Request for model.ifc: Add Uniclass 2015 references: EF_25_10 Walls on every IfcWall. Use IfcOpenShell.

First a look at what the model holds.

```python
import ifcopenshell

model = ifcopenshell.open("model.ifc")
print(model.schema)
print("classifications:", [c.Name for c in model.by_type("IfcClassification")])
for ifc_class in ("IfcDoor", "IfcRoof", "IfcStair", "IfcWall", "IfcWindow"):
    print(ifc_class, len(model.by_type(ifc_class)))
```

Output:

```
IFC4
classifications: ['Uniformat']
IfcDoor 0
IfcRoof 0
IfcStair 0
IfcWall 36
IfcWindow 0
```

```python
import ifcopenshell
import ifcopenshell.api.classification

model = ifcopenshell.open("model.ifc")

system = ifcopenshell.api.classification.add_classification(model, classification="Uniclass 2015")

codes = {
    "IfcWall": ("EF_25_10", "Walls"),
}
for ifc_class, (code, name) in codes.items():
    products = model.by_type(ifc_class)
    ifcopenshell.api.classification.add_reference(
        model, products=products, classification=system, identification=code, name=name
    )
    print(code, len(products))

model.write("model_v2.ifc")
```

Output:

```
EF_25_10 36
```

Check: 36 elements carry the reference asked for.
